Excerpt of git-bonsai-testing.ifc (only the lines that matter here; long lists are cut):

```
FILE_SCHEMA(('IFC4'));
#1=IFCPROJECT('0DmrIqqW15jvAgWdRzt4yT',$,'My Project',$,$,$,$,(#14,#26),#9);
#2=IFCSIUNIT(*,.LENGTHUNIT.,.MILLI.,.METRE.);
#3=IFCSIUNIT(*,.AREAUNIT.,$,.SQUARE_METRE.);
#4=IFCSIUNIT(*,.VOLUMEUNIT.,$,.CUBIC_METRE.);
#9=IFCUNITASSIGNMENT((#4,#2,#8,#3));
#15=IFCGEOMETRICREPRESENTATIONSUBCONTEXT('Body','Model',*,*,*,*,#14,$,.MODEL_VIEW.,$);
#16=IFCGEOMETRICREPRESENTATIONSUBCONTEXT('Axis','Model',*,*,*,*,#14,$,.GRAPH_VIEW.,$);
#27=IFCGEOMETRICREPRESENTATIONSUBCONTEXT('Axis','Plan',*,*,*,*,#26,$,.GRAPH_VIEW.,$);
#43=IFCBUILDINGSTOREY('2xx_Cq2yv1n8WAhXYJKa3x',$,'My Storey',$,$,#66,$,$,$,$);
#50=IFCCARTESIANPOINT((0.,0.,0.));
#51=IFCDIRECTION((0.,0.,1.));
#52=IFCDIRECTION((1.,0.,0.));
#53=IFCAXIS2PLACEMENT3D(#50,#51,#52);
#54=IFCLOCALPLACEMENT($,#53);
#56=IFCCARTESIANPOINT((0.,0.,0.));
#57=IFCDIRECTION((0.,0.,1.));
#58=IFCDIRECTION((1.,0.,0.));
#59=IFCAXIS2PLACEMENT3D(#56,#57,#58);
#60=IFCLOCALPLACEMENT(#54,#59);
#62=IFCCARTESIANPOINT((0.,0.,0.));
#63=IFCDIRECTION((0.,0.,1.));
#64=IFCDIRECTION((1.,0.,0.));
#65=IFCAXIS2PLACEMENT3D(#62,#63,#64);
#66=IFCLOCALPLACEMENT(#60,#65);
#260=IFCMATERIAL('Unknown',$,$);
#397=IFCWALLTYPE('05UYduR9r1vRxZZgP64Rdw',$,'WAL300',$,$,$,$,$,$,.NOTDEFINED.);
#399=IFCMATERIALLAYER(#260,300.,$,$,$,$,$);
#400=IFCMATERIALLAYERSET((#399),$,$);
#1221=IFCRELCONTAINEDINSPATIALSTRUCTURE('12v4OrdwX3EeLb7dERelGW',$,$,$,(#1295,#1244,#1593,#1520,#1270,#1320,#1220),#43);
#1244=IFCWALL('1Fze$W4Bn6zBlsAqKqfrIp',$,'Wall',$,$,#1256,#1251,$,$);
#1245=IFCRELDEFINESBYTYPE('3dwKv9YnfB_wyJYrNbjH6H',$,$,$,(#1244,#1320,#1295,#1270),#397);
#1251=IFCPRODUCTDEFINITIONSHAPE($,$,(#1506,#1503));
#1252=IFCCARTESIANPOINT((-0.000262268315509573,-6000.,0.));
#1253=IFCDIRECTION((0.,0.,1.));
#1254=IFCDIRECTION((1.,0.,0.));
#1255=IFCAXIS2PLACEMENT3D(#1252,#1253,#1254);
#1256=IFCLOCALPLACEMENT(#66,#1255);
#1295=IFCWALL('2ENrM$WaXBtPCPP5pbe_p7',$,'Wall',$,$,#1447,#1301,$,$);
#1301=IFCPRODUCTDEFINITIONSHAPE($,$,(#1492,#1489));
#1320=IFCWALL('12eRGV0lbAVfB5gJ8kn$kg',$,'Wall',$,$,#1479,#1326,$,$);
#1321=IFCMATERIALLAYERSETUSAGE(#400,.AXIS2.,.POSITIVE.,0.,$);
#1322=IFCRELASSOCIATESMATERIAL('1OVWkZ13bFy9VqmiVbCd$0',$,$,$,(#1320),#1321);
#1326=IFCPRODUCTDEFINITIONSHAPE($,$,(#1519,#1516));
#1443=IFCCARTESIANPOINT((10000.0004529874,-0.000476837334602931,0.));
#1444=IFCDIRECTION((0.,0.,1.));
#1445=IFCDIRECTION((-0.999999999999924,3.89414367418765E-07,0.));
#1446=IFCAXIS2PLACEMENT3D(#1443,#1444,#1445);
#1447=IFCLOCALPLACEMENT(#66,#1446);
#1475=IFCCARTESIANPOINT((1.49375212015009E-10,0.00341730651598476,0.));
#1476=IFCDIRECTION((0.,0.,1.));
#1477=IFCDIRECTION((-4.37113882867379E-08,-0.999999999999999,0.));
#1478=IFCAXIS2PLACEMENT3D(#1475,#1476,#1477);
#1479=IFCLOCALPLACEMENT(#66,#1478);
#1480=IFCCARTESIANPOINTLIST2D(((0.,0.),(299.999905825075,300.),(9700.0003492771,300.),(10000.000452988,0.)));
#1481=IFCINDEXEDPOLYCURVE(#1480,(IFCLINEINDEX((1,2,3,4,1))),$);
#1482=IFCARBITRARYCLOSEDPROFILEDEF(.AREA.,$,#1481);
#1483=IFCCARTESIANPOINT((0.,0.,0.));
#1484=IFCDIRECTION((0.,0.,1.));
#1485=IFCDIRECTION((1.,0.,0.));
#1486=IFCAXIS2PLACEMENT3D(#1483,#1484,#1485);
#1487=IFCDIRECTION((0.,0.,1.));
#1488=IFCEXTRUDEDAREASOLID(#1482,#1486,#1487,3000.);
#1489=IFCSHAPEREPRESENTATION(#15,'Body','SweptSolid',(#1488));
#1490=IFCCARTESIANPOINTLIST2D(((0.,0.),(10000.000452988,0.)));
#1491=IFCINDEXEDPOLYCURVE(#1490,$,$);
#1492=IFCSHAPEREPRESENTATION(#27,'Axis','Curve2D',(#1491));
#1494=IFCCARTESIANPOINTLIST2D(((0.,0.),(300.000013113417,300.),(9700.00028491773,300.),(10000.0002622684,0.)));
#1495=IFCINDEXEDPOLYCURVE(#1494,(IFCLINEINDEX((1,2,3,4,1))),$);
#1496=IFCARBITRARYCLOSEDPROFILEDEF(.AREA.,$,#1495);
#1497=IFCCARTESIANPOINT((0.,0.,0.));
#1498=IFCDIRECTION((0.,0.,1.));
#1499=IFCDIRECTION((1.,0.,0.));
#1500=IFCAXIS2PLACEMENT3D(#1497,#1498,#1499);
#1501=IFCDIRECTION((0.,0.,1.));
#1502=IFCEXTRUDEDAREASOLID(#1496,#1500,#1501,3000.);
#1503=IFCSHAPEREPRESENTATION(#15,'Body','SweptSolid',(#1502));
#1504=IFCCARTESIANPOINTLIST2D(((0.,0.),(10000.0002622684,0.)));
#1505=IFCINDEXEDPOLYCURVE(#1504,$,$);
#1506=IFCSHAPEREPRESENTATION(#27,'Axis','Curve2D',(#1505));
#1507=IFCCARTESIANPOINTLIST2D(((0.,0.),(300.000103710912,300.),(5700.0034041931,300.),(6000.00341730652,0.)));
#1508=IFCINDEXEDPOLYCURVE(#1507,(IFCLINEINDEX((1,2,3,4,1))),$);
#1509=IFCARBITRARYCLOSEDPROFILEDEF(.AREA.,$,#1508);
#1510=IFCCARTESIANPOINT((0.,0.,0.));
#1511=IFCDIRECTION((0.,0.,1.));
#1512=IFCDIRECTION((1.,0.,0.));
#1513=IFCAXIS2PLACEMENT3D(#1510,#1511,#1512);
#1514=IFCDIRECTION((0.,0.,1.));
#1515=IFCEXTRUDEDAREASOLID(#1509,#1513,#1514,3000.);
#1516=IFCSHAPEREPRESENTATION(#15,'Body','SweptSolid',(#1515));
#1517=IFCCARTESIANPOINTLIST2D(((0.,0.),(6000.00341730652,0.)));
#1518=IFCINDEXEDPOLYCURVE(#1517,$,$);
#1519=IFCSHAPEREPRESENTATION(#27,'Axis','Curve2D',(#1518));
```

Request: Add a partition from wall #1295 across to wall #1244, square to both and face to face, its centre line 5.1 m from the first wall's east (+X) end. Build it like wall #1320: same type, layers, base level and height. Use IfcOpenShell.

```python
import numpy as np
import ifcopenshell
import ifcopenshell.api.geometry
import ifcopenshell.api.material
import ifcopenshell.api.pset
import ifcopenshell.api.root
import ifcopenshell.api.spatial
import ifcopenshell.api.type
import ifcopenshell.geom
import ifcopenshell.util.element
import ifcopenshell.util.placement
import ifcopenshell.util.representation
import ifcopenshell.util.shape
import ifcopenshell.util.unit

model = ifcopenshell.open("git-bonsai-testing.ifc")
unit_scale = ifcopenshell.util.unit.calculate_unit_scale(model)
settings = ifcopenshell.geom.settings()
settings.set("use-world-coords", True)

start_wall = model.by_id(1295)
end_wall = model.by_guid("1Fze$W4Bn6zBlsAqKqfrIp")
like = model.by_guid("12eRGV0lbAVfB5gJ8kn$kg")
matrix = ifcopenshell.util.placement.get_local_placement(start_wall.ObjectPlacement)
matrix[:3, 3] *= unit_scale


def extent(element):
    """Bounding box in the first wall's axes, in metres."""
    shape = ifcopenshell.geom.create_shape(settings, element)
    points = (ifcopenshell.util.shape.get_vertices(shape.geometry) - matrix[:3, 3]) @ matrix[:3, :3]
    return points.min(axis=0), points.max(axis=0)


y_start = extent(start_wall)[1][1]
y_end = extent(end_wall)[0][1]
like_min, like_max = extent(like)
length, height = float(abs(y_end - y_start)), float(like_max[2] - like_min[2])
layer_set = ifcopenshell.util.element.get_material(like, should_skip_usage=True)
thickness = sum(layer.LayerThickness for layer in layer_set.MaterialLayers) * unit_scale

wall = ifcopenshell.api.root.create_entity(model, ifc_class="IfcWall", name="New partition")
storey = ifcopenshell.util.element.get_container(like)
ifcopenshell.api.spatial.assign_container(model, products=[wall], relating_structure=storey)
ifcopenshell.api.type.assign_type(
    model, related_objects=[wall], relating_type=ifcopenshell.util.element.get_type(like), should_map_representations=False
)
rel = ifcopenshell.api.material.assign_material(
    model, products=[wall], type="IfcMaterialLayerSetUsage", material=layer_set
)
rel.RelatingMaterial.OffsetFromReferenceLine = -thickness / 2 / unit_scale
pset = ifcopenshell.api.pset.add_pset(model, product=wall, name="Pset_WallCommon")
ifcopenshell.api.pset.edit_pset(model, pset=pset, properties={"IsExternal": False, "LoadBearing": False})

# The axis runs down the middle of the wall.
axis = ifcopenshell.api.geometry.add_axis_representation(
    model, context=ifcopenshell.util.representation.get_context(model, "Model", "Axis"), axis=[(0.0, 0.0), (length, 0.0)]
)
body = ifcopenshell.api.geometry.add_wall_representation(
    model,
    context=ifcopenshell.util.representation.get_context(model, "Model", "Body", "MODEL_VIEW"),
    length=length,
    height=height,
    thickness=thickness,
    offset=-thickness / 2,
)
for representation in (axis, body):
    ifcopenshell.api.geometry.assign_representation(model, product=wall, representation=representation)

placement = matrix @ ifcopenshell.util.placement.rotation(90, "Z")
placement[:, 3] = matrix @ np.array([extent(start_wall)[0][0] + 5.1, y_start, like_min[2], 1.0])
ifcopenshell.api.geometry.edit_object_placement(model, product=wall, matrix=placement)

print(f"partition {length:.3f} m long, {height:.3f} m high, {thickness:.3f} m thick")

model.write("git-bonsai-testing_updated.ifc")
```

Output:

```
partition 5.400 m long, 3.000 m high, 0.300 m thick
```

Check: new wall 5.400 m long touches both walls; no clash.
